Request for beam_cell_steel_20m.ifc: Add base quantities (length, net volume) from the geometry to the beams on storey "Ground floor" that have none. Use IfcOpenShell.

First a look at what the model holds.

```python
import ifcopenshell
import ifcopenshell.util.element
import ifcopenshell.util.unit

model = ifcopenshell.open("beam_cell_steel_20m.ifc")
print(model.schema)
for unit_type in ("LENGTHUNIT", "AREAUNIT", "VOLUMEUNIT"):
    print(unit_type, ifcopenshell.util.unit.calculate_unit_scale(model, unit_type))
storey = next(s for s in model.by_type("IfcBuildingStorey") if s.Name == "Ground floor")
beams = [e for e in ifcopenshell.util.element.get_decomposition(storey) if e.is_a("IfcBeam")]
for e in sorted(beams, key=lambda e: e.id()):
    print(e.id(), e.is_a(), e.Name, list(ifcopenshell.util.element.get_psets(e, qtos_only=True)), sep=" | ")
```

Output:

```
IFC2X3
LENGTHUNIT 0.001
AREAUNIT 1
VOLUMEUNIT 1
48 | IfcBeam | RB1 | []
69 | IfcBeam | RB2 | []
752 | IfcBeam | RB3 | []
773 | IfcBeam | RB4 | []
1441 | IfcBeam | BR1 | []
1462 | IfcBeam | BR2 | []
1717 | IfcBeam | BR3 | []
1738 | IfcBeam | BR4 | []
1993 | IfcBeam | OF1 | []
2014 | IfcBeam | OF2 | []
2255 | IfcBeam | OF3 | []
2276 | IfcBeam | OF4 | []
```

```python
import ifcopenshell
import ifcopenshell.api.pset
import ifcopenshell.geom
import ifcopenshell.util.element
import ifcopenshell.util.shape
import ifcopenshell.util.unit

model = ifcopenshell.open("beam_cell_steel_20m.ifc")
unit_scale = ifcopenshell.util.unit.calculate_unit_scale(model)
volume_scale = ifcopenshell.util.unit.calculate_unit_scale(model, "VOLUMEUNIT")
settings = ifcopenshell.geom.settings()

storey = next(s for s in model.by_type("IfcBuildingStorey") if s.Name == "Ground floor")
beams = [e for e in ifcopenshell.util.element.get_decomposition(storey) if e.is_a("IfcBeam")]

for e in sorted(beams, key=lambda e: e.id()):
    if ifcopenshell.util.element.get_psets(e, qtos_only=True, should_inherit=False):
        continue
    # Geometry comes back in metres, in the element's own axes.
    shape = ifcopenshell.geom.create_shape(settings, e)
    values = {
        "Length": ifcopenshell.util.shape.get_max_xyz(shape.geometry) / unit_scale,
        "NetVolume": ifcopenshell.util.shape.get_volume(shape.geometry) / volume_scale,
    }
    qto = ifcopenshell.api.pset.add_qto(model, product=e, name="BaseQuantities")
    ifcopenshell.api.pset.edit_qto(model, qto=qto, properties=values)
    print(e.id(), {k: round(v, 3) for k, v in values.items()})

model.write("beam_cell_steel_20m_updated.ifc")
```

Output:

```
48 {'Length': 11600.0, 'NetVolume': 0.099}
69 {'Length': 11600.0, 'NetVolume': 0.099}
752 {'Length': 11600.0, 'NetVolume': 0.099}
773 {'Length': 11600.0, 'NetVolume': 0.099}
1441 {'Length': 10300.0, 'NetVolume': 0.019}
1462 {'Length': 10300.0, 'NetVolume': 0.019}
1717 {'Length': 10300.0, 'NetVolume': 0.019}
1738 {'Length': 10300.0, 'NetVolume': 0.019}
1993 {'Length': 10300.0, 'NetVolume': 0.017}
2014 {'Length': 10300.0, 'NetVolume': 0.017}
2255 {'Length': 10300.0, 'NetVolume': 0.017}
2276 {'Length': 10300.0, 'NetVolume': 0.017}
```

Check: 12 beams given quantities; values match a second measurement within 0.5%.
